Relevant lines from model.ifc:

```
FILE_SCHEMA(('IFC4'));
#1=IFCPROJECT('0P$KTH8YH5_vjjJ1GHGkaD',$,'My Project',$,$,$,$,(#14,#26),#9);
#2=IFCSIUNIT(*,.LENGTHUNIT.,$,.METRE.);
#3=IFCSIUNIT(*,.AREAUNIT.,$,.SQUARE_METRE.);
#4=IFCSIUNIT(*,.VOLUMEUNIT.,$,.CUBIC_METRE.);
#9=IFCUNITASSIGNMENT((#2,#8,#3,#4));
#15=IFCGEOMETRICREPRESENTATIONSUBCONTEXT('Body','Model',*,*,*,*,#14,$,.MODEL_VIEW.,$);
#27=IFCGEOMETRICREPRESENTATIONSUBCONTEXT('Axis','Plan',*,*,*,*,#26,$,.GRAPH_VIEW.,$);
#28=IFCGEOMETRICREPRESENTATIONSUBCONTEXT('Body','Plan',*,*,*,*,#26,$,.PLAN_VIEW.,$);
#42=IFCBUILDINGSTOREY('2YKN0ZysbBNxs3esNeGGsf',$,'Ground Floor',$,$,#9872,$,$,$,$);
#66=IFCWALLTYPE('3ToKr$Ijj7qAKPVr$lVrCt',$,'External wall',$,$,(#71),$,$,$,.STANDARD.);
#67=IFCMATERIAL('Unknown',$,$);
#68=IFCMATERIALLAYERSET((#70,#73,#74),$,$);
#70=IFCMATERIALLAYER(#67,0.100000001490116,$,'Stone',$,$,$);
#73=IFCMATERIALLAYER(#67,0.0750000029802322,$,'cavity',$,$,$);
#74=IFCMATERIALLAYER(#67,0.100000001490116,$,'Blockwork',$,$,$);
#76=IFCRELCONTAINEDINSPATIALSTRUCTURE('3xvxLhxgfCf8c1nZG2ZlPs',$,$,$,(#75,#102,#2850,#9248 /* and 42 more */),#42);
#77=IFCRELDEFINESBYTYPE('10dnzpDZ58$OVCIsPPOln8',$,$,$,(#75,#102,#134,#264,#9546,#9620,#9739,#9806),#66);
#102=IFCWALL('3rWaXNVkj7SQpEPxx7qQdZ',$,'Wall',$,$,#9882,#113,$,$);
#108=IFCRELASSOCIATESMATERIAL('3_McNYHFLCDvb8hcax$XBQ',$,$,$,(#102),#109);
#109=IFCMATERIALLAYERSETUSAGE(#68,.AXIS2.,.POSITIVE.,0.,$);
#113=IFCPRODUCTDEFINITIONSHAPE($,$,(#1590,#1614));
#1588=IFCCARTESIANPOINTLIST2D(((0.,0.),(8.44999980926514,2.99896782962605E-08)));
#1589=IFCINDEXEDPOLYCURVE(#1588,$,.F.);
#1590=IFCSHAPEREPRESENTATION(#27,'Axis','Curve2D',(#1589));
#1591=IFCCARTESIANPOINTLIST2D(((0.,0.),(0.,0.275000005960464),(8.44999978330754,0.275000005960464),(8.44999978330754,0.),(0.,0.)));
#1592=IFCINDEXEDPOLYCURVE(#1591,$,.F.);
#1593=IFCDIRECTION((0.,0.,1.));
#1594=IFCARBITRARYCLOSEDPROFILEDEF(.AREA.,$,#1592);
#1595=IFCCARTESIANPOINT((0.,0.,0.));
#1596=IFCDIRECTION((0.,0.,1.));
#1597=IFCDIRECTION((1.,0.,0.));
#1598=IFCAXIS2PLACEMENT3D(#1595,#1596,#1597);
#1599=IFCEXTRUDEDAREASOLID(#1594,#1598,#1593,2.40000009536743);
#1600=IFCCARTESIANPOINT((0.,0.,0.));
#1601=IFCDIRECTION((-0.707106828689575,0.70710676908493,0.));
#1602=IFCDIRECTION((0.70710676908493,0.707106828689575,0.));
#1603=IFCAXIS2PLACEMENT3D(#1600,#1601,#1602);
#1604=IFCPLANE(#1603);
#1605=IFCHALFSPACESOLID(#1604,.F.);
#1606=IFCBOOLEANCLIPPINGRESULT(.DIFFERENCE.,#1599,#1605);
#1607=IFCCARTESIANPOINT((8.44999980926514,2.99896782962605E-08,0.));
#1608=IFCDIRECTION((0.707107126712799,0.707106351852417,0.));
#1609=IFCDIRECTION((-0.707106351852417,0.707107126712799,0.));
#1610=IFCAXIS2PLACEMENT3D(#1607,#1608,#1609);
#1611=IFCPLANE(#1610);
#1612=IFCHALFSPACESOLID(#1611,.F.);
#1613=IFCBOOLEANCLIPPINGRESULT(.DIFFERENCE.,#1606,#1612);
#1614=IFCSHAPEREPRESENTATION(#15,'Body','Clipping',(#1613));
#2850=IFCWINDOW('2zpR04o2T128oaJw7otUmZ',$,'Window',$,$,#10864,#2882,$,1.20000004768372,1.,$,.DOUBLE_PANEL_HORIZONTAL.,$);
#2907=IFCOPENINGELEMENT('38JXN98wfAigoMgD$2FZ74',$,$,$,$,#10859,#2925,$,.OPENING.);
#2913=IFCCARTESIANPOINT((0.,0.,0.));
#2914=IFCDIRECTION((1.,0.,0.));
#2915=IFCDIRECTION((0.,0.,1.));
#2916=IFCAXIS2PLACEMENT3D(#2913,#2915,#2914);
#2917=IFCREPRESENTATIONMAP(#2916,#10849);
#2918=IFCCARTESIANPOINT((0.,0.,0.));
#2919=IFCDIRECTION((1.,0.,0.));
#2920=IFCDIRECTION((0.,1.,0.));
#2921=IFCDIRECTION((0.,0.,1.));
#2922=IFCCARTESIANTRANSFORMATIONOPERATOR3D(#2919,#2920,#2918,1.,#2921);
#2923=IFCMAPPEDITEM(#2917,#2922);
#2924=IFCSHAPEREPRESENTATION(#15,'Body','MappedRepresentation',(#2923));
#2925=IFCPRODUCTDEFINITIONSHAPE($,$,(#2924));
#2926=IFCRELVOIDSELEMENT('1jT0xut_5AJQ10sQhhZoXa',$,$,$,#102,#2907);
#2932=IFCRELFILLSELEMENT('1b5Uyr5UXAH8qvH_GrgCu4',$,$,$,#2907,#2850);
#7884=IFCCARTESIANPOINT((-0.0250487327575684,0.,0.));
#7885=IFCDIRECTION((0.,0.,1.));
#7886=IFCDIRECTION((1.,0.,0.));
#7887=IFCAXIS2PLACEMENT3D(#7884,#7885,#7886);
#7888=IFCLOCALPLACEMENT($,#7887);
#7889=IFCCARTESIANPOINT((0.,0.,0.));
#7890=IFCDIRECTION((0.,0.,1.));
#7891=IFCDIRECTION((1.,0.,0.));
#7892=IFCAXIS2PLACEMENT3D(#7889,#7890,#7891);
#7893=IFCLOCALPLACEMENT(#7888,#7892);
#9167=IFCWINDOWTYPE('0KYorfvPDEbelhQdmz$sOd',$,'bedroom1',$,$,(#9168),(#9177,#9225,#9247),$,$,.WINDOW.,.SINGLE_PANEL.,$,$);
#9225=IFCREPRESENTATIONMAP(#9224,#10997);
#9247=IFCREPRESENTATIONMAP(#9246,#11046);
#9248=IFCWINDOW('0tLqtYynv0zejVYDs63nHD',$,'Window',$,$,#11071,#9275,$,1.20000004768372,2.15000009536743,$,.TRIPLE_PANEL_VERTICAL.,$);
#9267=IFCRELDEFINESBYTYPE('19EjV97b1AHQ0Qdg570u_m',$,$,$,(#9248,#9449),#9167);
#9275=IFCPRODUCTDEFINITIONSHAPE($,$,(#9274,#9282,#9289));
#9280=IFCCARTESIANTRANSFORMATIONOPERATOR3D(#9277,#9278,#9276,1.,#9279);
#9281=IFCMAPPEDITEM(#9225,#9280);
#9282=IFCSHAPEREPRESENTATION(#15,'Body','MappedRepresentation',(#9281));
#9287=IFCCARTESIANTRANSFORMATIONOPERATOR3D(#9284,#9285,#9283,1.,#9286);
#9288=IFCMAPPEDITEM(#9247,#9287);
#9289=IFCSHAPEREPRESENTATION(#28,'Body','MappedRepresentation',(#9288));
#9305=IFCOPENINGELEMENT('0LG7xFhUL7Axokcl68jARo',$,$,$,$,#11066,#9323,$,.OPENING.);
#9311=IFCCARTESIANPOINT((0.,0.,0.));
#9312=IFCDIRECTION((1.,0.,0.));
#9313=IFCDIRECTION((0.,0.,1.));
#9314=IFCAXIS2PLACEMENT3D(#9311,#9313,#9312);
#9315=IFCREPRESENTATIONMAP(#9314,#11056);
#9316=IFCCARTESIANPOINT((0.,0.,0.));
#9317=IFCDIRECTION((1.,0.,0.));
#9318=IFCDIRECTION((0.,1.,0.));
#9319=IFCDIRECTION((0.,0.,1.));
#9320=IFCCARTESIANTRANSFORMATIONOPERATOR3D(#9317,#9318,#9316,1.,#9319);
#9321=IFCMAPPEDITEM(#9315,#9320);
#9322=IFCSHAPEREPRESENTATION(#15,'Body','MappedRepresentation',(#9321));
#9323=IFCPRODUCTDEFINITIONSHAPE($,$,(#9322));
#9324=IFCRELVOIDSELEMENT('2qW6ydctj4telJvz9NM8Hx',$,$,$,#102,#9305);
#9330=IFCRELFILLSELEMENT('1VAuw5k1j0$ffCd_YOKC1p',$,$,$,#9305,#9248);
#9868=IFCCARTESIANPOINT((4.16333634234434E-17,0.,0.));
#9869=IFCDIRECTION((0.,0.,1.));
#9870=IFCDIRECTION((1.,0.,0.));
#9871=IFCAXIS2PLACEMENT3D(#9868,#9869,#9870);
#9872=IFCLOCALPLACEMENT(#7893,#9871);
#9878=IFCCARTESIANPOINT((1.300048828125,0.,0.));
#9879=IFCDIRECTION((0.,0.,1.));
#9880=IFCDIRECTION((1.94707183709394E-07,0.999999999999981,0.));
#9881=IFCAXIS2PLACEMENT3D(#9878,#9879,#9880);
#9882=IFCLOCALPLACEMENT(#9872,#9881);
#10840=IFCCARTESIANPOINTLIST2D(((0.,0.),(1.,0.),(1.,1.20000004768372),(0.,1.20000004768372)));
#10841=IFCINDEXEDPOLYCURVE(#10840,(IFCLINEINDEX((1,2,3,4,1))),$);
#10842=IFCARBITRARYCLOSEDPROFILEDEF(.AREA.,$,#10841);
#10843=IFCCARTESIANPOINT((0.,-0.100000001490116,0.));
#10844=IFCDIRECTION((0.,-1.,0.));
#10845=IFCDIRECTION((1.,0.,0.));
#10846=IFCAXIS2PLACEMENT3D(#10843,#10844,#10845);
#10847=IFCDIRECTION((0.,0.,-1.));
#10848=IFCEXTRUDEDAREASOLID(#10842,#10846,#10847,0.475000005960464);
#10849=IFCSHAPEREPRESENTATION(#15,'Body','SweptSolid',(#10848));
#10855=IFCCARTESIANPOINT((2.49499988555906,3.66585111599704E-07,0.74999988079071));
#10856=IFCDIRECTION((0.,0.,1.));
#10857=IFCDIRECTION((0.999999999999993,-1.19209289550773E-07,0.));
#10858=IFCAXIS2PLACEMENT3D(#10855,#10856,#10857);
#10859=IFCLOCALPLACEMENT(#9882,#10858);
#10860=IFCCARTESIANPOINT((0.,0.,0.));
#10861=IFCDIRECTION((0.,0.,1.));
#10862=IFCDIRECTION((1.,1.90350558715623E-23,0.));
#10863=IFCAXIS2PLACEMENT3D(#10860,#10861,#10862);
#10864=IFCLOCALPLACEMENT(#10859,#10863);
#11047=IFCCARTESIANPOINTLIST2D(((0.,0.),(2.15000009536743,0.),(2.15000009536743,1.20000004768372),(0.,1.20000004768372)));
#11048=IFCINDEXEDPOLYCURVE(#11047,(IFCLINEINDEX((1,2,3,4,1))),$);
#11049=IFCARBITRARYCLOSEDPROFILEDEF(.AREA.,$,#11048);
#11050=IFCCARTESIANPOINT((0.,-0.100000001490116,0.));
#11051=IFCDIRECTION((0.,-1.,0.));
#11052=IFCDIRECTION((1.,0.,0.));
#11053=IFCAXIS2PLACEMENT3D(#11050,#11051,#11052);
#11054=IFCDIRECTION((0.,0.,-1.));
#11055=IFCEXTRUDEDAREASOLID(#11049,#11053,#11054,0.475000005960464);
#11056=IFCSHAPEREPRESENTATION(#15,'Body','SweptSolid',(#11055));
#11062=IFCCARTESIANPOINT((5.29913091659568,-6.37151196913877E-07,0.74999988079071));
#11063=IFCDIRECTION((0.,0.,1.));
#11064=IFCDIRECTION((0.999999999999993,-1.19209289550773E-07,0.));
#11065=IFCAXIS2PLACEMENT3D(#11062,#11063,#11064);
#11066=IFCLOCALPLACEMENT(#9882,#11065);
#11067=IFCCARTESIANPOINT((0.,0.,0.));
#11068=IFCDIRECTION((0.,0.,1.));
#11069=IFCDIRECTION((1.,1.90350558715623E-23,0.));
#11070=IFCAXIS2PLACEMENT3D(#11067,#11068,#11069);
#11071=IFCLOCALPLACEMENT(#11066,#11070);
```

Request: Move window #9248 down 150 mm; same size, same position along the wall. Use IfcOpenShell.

```python
import numpy as np
import ifcopenshell
import ifcopenshell.api.geometry
import ifcopenshell.util.placement
import ifcopenshell.util.unit

model = ifcopenshell.open("model.ifc")
unit_scale = ifcopenshell.util.unit.calculate_unit_scale(model)

window = model.by_guid("0tLqtYynv0zejVYDs63nHD")
opening = window.FillsVoids[0].RelatingOpeningElement
dz = -0.15 / unit_scale

shift = np.array([0.0, 0.0, dz])
# The window is placed relative to its opening, so it follows when the opening moves.
matrix = ifcopenshell.util.placement.get_local_placement(opening.ObjectPlacement)
matrix[:3, 3] += shift
ifcopenshell.api.geometry.edit_object_placement(
    model, product=opening, matrix=matrix, is_si=False, should_transform_children=True
)

print(f"moved by {dz * unit_scale:+.3f} m")

model.write("model_edited.ifc")
```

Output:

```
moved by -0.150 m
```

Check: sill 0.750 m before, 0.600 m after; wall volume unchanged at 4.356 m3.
